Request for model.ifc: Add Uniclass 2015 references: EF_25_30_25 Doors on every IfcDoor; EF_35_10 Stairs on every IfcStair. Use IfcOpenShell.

First a look at what the model holds.

```python
import ifcopenshell

model = ifcopenshell.open("model.ifc")
print(model.schema)
print("classifications:", [c.Name for c in model.by_type("IfcClassification")])
for ifc_class in ("IfcDoor", "IfcRoof", "IfcStair", "IfcWall", "IfcWindow"):
    print(ifc_class, len(model.by_type(ifc_class)))
```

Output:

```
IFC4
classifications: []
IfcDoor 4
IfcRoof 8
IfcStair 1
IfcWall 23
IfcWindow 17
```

```python
import ifcopenshell
import ifcopenshell.api.classification

model = ifcopenshell.open("model.ifc")

system = ifcopenshell.api.classification.add_classification(model, classification="Uniclass 2015")

codes = {
    "IfcDoor": ("EF_25_30_25", "Doors"),
    "IfcStair": ("EF_35_10", "Stairs"),
}
for ifc_class, (code, name) in codes.items():
    products = model.by_type(ifc_class)
    ifcopenshell.api.classification.add_reference(
        model, products=products, classification=system, identification=code, name=name
    )
    print(code, len(products))

model.write("model_updated.ifc")
```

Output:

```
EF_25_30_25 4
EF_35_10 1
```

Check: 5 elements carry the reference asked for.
